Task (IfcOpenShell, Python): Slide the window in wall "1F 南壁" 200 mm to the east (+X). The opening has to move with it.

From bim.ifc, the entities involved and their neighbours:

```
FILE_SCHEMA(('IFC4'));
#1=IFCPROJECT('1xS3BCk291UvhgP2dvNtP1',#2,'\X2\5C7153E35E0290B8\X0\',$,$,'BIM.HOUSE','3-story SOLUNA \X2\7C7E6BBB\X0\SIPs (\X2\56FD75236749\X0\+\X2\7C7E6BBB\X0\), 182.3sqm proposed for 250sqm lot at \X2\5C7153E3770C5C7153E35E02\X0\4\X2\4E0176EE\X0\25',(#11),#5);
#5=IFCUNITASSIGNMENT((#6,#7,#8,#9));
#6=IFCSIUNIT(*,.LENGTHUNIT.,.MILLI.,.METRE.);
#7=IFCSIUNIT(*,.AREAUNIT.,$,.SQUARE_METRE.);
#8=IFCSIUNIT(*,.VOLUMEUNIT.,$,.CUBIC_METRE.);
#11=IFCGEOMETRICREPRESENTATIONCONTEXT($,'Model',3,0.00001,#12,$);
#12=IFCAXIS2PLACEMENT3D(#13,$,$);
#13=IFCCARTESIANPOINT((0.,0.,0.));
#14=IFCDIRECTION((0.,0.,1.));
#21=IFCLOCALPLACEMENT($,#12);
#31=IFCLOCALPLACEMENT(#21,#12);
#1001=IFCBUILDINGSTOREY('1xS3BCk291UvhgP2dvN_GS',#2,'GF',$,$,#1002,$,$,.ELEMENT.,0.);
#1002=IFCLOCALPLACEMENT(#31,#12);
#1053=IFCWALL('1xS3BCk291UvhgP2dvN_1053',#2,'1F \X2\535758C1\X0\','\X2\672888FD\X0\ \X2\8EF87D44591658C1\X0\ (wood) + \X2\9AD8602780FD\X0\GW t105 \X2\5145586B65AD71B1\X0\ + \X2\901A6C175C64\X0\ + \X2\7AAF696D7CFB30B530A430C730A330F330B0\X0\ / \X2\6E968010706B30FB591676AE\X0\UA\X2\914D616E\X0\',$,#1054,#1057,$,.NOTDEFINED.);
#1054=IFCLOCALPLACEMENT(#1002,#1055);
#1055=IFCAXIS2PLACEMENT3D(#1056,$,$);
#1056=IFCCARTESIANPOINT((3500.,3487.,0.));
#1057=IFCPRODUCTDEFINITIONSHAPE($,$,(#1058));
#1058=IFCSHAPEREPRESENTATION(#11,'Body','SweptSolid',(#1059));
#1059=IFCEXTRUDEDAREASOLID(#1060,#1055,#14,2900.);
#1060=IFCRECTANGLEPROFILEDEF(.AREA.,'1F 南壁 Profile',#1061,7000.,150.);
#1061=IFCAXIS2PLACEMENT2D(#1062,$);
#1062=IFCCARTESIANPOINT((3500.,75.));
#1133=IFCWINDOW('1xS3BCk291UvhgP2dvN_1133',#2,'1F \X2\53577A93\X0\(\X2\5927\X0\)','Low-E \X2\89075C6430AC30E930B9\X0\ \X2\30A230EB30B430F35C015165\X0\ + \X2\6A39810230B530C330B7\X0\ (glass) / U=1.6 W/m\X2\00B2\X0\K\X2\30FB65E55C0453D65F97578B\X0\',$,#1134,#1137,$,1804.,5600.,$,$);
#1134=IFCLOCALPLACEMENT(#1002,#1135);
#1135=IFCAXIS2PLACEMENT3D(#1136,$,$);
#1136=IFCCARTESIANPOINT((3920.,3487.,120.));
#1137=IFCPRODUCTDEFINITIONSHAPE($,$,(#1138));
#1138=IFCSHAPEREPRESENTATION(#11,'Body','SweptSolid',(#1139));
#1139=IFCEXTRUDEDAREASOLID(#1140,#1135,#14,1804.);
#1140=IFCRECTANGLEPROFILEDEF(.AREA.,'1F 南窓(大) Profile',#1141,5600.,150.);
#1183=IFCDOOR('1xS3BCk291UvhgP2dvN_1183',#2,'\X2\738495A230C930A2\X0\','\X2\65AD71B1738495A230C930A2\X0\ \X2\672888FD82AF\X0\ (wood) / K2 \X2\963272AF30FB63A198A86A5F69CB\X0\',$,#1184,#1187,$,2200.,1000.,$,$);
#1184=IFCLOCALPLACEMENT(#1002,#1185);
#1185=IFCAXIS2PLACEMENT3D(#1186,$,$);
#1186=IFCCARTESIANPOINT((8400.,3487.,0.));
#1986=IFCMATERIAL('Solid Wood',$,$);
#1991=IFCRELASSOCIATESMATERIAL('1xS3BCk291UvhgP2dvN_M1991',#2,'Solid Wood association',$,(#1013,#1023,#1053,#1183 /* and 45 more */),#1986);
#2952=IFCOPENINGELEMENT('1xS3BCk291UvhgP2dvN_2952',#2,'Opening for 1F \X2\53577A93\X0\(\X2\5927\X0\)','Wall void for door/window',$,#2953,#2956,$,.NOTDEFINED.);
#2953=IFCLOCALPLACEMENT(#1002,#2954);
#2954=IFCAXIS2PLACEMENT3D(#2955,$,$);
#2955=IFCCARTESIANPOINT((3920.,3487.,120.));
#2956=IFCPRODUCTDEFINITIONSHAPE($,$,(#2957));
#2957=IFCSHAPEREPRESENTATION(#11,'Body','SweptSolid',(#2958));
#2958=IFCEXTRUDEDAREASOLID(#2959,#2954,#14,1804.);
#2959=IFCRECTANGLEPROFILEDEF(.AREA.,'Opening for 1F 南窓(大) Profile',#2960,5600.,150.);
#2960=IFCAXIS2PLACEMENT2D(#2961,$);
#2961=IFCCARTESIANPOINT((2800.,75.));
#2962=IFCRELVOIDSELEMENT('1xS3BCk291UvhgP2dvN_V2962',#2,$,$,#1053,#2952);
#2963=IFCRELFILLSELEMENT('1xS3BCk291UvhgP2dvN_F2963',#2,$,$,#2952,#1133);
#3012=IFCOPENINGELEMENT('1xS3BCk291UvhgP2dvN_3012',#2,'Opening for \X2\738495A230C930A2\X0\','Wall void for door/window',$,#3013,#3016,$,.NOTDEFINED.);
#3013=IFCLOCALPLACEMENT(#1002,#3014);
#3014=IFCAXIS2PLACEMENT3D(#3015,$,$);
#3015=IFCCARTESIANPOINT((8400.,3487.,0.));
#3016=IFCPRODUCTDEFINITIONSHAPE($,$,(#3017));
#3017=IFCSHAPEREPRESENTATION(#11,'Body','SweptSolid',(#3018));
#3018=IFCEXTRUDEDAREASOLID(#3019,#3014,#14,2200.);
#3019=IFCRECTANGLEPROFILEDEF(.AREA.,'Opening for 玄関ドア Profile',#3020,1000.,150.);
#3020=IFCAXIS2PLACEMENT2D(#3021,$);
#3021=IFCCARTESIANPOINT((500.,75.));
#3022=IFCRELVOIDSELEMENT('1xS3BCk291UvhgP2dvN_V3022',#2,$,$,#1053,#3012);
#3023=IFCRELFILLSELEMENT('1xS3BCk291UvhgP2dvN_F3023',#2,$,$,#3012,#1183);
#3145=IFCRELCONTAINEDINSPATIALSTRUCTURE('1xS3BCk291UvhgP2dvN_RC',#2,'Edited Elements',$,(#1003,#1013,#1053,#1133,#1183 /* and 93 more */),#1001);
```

```python
import ifcopenshell
import ifcopenshell.api.geometry
import ifcopenshell.util.placement
import ifcopenshell.util.unit

model = ifcopenshell.open("bim.ifc")
unit_scale = ifcopenshell.util.unit.calculate_unit_scale(model)

window = model.by_id(1133)
opening = window.FillsVoids[0].RelatingOpeningElement
wall = opening.VoidsElements[0].RelatingBuildingElement

wall_matrix = ifcopenshell.util.placement.get_local_placement(wall.ObjectPlacement)
shift = wall_matrix[:3, 0] * 0.2 / unit_scale
before = ifcopenshell.util.placement.get_local_placement(window.ObjectPlacement)[:3, 3].copy()

# The window is not placed relative to its opening, so move both.
for product in (opening, window):
    matrix = ifcopenshell.util.placement.get_local_placement(product.ObjectPlacement)
    matrix[:3, 3] += shift
    ifcopenshell.api.geometry.edit_object_placement(model, product=product, matrix=matrix, is_si=False)

after = ifcopenshell.util.placement.get_local_placement(window.ObjectPlacement)[:3, 3]
print("window moved by", (after - before).round(3) + 0.0)

model.write("bim-out.ifc")
```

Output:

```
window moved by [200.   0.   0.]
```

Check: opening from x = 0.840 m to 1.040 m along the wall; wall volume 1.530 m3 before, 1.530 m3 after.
